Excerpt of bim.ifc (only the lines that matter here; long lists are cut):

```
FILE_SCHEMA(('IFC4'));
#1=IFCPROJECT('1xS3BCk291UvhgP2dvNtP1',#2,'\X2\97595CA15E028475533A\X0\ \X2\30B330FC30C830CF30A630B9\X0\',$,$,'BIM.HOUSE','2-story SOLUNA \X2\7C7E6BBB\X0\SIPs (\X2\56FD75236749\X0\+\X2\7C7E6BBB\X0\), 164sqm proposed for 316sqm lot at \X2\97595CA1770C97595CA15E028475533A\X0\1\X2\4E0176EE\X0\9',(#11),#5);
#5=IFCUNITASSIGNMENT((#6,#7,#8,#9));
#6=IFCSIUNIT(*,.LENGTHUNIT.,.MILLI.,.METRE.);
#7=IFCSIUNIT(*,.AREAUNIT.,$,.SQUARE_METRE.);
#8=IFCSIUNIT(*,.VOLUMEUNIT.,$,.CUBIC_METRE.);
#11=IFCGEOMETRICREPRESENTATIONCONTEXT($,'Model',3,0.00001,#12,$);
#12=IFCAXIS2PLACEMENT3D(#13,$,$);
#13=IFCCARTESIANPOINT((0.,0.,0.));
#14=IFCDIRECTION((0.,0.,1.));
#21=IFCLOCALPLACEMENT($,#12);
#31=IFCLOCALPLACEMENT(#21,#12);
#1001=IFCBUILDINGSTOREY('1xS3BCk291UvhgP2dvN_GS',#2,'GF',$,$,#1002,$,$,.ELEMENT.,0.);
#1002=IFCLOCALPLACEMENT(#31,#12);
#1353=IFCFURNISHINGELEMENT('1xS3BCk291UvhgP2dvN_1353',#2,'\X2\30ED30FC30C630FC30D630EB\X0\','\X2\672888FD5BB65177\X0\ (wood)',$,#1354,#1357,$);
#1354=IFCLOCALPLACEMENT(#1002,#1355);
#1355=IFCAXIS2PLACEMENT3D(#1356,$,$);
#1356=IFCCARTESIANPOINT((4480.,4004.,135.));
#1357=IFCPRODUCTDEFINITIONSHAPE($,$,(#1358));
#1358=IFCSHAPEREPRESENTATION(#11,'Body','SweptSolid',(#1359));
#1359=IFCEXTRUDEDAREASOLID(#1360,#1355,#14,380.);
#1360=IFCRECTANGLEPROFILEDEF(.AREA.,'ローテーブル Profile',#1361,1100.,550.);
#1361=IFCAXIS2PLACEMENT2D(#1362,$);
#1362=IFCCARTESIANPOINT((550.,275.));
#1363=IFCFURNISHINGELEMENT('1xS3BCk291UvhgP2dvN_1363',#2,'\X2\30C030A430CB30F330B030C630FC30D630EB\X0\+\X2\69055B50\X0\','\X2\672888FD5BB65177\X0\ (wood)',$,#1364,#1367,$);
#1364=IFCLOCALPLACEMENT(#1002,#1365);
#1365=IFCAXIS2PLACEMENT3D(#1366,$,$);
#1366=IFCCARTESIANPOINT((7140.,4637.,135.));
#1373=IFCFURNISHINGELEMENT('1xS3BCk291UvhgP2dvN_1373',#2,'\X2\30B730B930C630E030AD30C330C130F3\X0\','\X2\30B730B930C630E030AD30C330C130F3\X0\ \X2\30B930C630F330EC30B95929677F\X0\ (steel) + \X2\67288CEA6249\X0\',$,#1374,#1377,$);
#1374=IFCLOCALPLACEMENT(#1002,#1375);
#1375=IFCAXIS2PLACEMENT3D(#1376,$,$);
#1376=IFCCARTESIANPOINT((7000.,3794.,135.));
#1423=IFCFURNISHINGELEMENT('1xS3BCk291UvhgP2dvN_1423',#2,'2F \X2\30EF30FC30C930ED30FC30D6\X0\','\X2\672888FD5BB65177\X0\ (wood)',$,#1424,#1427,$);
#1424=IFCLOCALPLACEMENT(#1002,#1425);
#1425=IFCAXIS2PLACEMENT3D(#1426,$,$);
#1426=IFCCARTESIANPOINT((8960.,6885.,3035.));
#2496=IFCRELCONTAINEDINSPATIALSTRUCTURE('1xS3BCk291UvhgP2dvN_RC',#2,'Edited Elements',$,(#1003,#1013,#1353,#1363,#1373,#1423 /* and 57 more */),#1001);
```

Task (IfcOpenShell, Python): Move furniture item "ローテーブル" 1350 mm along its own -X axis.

```python
import ifcopenshell
import ifcopenshell.api.geometry
import ifcopenshell.util.placement

model = ifcopenshell.open("bim.ifc")

item = model.by_id(1353)
matrix = ifcopenshell.util.placement.get_local_placement(item.ObjectPlacement)
matrix[:3, 3] -= matrix[:3, 0] * 1350.0
ifcopenshell.api.geometry.edit_object_placement(model, product=item, matrix=matrix, is_si=False)

print(ifcopenshell.util.placement.get_local_placement(item.ObjectPlacement).round(3) + 0.0)

model.write("bim_v2.ifc")
```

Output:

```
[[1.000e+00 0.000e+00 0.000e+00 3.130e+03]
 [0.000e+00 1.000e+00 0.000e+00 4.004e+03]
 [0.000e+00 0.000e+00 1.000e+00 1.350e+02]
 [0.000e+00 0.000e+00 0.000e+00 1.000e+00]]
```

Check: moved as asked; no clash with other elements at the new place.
